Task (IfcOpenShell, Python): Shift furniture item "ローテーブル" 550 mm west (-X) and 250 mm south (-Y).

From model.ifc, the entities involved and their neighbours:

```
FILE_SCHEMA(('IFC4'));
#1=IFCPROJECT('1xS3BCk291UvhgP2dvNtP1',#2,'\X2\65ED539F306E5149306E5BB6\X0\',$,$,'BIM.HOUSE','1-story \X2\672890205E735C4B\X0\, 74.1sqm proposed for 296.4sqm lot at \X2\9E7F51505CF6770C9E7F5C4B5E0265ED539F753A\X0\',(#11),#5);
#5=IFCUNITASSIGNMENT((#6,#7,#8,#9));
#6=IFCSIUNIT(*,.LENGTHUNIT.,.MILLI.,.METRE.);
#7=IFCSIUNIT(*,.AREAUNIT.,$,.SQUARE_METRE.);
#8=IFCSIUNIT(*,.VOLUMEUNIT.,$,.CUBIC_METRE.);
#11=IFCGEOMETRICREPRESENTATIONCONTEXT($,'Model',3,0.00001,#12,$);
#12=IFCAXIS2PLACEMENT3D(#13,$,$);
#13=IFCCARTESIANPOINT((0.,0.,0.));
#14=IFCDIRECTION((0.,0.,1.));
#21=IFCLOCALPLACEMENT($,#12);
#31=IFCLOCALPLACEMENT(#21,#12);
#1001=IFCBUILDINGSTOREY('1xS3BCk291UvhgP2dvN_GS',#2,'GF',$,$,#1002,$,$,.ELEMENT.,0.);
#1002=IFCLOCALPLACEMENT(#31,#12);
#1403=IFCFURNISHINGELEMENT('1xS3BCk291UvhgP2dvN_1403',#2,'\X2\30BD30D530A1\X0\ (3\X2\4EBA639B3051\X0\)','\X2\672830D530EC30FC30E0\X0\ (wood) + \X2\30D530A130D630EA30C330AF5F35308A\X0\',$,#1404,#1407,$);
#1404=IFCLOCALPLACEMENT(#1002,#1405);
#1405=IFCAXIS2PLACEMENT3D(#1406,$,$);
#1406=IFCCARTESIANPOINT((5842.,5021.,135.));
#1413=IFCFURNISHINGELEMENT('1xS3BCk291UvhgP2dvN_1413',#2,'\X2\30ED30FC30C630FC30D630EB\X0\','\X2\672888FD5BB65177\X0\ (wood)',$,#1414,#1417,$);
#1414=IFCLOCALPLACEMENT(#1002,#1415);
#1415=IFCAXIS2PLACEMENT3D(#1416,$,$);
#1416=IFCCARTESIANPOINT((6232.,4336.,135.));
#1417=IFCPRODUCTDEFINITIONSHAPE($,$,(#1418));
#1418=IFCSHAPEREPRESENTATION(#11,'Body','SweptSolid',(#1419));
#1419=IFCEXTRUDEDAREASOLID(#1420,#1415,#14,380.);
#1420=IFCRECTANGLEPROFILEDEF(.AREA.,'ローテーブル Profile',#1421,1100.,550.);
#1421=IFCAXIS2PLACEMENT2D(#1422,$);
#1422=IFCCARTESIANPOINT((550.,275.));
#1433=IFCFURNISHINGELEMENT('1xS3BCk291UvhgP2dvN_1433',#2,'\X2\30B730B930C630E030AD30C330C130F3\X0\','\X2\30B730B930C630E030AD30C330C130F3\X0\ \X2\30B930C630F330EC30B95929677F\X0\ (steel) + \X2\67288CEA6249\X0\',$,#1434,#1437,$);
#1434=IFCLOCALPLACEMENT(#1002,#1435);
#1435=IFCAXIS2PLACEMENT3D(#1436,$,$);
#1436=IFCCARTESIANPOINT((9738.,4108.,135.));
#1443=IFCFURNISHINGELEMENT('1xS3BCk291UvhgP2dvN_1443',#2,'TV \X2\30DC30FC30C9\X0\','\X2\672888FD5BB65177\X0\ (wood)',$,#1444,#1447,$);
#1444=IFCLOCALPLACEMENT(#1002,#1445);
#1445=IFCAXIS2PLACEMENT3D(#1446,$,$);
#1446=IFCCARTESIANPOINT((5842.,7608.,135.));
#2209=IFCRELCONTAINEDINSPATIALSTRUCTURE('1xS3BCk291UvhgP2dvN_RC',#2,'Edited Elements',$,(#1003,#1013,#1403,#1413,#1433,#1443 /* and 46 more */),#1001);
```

```python
import ifcopenshell
import ifcopenshell.api.geometry
import ifcopenshell.util.placement

model = ifcopenshell.open("model.ifc")

item = model.by_guid("1xS3BCk291UvhgP2dvN_1413")
matrix = ifcopenshell.util.placement.get_local_placement(item.ObjectPlacement)
matrix[0, 3] -= 550.0
matrix[1, 3] -= 250.0
ifcopenshell.api.geometry.edit_object_placement(model, product=item, matrix=matrix, is_si=False)

print(ifcopenshell.util.placement.get_local_placement(item.ObjectPlacement).round(3) + 0.0)

model.write("model_v2.ifc")
```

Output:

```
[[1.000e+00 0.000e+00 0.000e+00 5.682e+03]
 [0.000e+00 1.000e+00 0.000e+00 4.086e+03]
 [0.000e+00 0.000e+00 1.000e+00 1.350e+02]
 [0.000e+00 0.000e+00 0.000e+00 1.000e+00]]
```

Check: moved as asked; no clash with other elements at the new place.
